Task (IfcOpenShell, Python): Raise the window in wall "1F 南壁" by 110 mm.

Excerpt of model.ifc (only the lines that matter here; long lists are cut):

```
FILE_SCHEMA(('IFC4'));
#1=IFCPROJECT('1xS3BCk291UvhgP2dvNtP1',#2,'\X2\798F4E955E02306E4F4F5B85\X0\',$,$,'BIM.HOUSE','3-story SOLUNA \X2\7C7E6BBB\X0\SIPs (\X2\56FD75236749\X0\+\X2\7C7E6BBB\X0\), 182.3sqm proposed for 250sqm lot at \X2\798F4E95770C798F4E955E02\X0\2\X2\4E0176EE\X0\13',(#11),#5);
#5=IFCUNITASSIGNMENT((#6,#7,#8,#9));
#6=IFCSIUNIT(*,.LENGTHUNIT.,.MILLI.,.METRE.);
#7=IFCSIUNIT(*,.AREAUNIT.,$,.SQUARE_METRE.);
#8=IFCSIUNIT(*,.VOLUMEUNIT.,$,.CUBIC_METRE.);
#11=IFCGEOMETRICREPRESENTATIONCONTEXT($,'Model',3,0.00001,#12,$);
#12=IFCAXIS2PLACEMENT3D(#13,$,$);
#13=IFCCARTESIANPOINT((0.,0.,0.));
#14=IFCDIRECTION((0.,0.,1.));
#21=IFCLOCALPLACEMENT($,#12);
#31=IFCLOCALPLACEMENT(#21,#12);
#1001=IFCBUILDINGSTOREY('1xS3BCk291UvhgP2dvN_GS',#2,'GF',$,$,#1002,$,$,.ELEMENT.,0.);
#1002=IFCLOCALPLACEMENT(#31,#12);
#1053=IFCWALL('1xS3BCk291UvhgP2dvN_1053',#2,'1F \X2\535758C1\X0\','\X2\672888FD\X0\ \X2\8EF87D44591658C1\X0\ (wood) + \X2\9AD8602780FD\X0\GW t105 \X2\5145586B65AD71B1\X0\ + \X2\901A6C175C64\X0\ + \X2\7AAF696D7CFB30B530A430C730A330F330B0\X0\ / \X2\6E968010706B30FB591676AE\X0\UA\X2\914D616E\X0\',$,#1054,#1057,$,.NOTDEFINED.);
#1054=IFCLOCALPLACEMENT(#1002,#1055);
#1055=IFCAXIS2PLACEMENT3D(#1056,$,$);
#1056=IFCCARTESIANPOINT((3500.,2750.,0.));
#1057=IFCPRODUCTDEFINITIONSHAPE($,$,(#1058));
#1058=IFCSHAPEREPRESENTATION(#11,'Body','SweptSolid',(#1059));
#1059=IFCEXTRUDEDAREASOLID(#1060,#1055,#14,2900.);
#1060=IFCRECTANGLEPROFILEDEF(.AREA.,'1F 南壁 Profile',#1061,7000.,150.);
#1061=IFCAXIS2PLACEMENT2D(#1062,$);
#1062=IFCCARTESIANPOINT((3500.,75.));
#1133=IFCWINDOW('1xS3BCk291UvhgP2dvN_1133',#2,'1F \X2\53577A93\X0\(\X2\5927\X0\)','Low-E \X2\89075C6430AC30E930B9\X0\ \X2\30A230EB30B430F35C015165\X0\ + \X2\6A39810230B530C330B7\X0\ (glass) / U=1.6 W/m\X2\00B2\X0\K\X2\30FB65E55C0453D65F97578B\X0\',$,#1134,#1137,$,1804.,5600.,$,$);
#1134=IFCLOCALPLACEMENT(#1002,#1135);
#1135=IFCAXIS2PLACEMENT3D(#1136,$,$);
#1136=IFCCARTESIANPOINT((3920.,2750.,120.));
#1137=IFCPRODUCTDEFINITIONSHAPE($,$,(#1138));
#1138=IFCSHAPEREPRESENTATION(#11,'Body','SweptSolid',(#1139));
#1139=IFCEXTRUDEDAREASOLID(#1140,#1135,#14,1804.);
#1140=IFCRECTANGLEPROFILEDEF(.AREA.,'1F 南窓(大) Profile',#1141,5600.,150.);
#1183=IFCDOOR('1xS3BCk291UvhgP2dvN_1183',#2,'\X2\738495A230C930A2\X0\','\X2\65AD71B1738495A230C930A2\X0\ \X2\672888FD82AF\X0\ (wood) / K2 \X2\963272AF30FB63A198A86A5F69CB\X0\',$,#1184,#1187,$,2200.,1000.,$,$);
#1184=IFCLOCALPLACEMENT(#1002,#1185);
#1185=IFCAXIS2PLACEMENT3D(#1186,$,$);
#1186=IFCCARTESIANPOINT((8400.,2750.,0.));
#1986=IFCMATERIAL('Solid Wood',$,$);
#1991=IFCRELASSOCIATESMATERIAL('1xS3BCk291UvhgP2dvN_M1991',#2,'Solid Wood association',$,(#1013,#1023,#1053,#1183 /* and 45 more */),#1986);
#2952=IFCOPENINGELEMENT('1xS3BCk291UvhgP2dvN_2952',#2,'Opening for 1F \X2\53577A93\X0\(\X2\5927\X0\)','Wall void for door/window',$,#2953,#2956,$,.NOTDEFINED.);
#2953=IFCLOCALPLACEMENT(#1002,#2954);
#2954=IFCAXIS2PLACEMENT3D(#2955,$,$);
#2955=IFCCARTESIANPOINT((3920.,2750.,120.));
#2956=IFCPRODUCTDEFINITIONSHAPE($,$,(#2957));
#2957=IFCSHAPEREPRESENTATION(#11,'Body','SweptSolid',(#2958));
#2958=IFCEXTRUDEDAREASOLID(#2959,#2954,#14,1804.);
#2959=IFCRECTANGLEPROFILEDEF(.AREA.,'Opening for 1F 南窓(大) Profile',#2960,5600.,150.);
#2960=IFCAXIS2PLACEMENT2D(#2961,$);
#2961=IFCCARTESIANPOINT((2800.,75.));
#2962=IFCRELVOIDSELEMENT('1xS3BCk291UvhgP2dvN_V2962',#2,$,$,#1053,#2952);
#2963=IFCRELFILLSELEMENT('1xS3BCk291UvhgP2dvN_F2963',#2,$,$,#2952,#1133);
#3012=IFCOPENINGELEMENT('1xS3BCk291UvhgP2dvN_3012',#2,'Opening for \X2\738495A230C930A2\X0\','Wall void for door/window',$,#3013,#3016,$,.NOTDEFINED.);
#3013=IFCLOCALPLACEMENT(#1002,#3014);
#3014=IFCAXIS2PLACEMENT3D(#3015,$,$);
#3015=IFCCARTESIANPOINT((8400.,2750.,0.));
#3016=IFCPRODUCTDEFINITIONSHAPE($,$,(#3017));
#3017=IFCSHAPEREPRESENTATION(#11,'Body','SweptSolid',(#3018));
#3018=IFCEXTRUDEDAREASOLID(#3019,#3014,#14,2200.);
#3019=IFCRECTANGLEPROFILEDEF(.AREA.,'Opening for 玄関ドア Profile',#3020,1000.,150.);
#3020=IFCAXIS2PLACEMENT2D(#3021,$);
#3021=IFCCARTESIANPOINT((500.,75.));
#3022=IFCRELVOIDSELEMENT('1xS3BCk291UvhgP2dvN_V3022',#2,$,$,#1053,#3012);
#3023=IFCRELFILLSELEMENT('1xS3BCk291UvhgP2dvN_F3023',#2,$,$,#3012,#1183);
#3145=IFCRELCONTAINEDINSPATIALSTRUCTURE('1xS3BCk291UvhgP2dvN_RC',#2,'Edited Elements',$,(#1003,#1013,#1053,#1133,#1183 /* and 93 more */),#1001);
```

```python
import numpy as np
import ifcopenshell
import ifcopenshell.api.geometry
import ifcopenshell.util.placement
import ifcopenshell.util.unit

model = ifcopenshell.open("model.ifc")
unit_scale = ifcopenshell.util.unit.calculate_unit_scale(model)

window = model.by_guid("1xS3BCk291UvhgP2dvN_1133")
opening = window.FillsVoids[0].RelatingOpeningElement
dz = 0.11 / unit_scale

shift = np.array([0.0, 0.0, dz])
# The window is not placed relative to its opening, so move both.
for product in (opening, window):
    matrix = ifcopenshell.util.placement.get_local_placement(product.ObjectPlacement)
    matrix[:3, 3] += shift
    ifcopenshell.api.geometry.edit_object_placement(model, product=product, matrix=matrix, is_si=False)

print(f"moved by {dz * unit_scale:+.3f} m")

model.write("model-out.ifc")
```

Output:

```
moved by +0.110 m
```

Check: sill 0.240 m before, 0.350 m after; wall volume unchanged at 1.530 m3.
